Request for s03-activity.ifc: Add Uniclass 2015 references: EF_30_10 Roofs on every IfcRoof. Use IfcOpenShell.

First a look at what the model holds.

```python
import ifcopenshell

model = ifcopenshell.open("s03-activity.ifc")
print(model.schema)
print("classifications:", [c.Name for c in model.by_type("IfcClassification")])
for ifc_class in ("IfcDoor", "IfcRoof", "IfcStair", "IfcWall", "IfcWindow"):
    print(ifc_class, len(model.by_type(ifc_class)))
```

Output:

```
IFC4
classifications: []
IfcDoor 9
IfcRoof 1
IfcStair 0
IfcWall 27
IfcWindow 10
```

```python
import ifcopenshell
import ifcopenshell.api.classification

model = ifcopenshell.open("s03-activity.ifc")

system = ifcopenshell.api.classification.add_classification(model, classification="Uniclass 2015")

codes = {
    "IfcRoof": ("EF_30_10", "Roofs"),
}
for ifc_class, (code, name) in codes.items():
    products = model.by_type(ifc_class)
    ifcopenshell.api.classification.add_reference(
        model, products=products, classification=system, identification=code, name=name
    )
    print(code, len(products))

model.write("s03-activity_updated.ifc")
```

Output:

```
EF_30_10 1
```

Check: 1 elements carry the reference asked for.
